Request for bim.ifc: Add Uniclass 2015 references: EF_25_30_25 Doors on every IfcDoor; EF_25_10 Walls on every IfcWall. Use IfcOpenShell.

First a look at what the model holds.

```python
import ifcopenshell

model = ifcopenshell.open("bim.ifc")
print(model.schema)
print("classifications:", [c.Name for c in model.by_type("IfcClassification")])
for ifc_class in ("IfcDoor", "IfcRoof", "IfcStair", "IfcWall", "IfcWindow"):
    print(ifc_class, len(model.by_type(ifc_class)))
```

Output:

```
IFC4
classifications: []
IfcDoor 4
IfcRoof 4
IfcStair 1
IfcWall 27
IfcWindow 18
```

```python
import ifcopenshell
import ifcopenshell.api.classification

model = ifcopenshell.open("bim.ifc")

system = ifcopenshell.api.classification.add_classification(model, classification="Uniclass 2015")

codes = {
    "IfcDoor": ("EF_25_30_25", "Doors"),
    "IfcWall": ("EF_25_10", "Walls"),
}
for ifc_class, (code, name) in codes.items():
    products = model.by_type(ifc_class)
    ifcopenshell.api.classification.add_reference(
        model, products=products, classification=system, identification=code, name=name
    )
    print(code, len(products))

model.write("bim-out.ifc")
```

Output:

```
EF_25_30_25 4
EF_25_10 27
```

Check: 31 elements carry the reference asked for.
